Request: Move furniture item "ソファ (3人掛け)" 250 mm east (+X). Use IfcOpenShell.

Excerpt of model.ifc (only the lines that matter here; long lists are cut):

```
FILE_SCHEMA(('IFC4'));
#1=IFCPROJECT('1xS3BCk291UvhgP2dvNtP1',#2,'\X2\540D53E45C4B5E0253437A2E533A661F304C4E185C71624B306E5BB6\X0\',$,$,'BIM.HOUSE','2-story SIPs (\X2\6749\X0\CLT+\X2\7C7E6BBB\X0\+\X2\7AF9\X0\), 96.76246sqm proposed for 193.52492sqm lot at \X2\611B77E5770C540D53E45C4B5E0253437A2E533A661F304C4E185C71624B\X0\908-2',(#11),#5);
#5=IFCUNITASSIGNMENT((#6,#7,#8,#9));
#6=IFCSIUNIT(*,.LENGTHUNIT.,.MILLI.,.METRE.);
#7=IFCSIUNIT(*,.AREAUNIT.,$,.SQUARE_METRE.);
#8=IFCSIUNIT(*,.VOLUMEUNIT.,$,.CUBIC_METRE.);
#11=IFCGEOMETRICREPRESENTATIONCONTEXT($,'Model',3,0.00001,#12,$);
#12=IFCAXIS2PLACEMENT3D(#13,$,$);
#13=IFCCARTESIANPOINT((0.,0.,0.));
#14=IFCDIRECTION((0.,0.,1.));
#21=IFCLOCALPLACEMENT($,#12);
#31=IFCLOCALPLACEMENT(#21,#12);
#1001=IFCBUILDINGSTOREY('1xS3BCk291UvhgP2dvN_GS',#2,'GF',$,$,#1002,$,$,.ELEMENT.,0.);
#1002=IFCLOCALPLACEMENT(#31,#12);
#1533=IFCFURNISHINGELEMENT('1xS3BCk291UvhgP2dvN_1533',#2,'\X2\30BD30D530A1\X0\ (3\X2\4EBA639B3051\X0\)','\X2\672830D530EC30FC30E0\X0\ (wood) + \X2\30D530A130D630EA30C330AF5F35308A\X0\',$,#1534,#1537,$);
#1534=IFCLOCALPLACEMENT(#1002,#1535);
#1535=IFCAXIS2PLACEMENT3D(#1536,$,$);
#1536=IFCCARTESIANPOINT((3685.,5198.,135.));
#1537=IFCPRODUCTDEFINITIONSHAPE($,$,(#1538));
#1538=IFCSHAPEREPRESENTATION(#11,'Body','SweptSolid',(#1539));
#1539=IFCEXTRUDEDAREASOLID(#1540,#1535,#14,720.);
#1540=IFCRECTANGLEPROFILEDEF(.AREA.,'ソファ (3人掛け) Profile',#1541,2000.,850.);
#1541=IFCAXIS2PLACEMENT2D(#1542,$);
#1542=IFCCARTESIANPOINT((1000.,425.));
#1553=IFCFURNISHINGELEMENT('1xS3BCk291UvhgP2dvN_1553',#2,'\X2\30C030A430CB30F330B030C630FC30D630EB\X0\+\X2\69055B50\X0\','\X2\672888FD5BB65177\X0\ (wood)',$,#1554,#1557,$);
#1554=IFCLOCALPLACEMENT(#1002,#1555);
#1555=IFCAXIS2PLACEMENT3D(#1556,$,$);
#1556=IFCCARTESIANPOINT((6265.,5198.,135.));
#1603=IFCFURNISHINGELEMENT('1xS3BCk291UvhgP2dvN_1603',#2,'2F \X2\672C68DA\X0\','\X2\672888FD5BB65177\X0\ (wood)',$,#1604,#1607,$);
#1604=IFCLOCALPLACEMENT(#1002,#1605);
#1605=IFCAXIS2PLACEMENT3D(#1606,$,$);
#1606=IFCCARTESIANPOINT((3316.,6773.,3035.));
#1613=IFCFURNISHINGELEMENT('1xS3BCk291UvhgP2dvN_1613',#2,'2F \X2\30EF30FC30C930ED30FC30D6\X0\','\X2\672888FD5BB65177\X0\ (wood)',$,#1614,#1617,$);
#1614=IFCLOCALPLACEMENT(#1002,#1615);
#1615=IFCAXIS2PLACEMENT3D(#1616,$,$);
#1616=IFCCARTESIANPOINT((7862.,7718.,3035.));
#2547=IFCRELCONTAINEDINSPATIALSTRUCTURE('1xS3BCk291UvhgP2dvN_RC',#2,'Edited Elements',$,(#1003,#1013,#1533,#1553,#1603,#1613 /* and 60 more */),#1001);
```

```python
import ifcopenshell
import ifcopenshell.api.geometry
import ifcopenshell.util.placement

model = ifcopenshell.open("model.ifc")

item = model.by_guid("1xS3BCk291UvhgP2dvN_1533")
matrix = ifcopenshell.util.placement.get_local_placement(item.ObjectPlacement)
matrix[0, 3] += 250.0
ifcopenshell.api.geometry.edit_object_placement(model, product=item, matrix=matrix, is_si=False)

print(ifcopenshell.util.placement.get_local_placement(item.ObjectPlacement).round(3) + 0.0)

model.write("model-out.ifc")
```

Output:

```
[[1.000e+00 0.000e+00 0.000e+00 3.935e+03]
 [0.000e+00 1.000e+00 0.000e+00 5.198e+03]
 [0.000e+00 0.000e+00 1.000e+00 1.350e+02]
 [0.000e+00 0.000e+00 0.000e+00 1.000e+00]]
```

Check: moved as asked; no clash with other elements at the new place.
